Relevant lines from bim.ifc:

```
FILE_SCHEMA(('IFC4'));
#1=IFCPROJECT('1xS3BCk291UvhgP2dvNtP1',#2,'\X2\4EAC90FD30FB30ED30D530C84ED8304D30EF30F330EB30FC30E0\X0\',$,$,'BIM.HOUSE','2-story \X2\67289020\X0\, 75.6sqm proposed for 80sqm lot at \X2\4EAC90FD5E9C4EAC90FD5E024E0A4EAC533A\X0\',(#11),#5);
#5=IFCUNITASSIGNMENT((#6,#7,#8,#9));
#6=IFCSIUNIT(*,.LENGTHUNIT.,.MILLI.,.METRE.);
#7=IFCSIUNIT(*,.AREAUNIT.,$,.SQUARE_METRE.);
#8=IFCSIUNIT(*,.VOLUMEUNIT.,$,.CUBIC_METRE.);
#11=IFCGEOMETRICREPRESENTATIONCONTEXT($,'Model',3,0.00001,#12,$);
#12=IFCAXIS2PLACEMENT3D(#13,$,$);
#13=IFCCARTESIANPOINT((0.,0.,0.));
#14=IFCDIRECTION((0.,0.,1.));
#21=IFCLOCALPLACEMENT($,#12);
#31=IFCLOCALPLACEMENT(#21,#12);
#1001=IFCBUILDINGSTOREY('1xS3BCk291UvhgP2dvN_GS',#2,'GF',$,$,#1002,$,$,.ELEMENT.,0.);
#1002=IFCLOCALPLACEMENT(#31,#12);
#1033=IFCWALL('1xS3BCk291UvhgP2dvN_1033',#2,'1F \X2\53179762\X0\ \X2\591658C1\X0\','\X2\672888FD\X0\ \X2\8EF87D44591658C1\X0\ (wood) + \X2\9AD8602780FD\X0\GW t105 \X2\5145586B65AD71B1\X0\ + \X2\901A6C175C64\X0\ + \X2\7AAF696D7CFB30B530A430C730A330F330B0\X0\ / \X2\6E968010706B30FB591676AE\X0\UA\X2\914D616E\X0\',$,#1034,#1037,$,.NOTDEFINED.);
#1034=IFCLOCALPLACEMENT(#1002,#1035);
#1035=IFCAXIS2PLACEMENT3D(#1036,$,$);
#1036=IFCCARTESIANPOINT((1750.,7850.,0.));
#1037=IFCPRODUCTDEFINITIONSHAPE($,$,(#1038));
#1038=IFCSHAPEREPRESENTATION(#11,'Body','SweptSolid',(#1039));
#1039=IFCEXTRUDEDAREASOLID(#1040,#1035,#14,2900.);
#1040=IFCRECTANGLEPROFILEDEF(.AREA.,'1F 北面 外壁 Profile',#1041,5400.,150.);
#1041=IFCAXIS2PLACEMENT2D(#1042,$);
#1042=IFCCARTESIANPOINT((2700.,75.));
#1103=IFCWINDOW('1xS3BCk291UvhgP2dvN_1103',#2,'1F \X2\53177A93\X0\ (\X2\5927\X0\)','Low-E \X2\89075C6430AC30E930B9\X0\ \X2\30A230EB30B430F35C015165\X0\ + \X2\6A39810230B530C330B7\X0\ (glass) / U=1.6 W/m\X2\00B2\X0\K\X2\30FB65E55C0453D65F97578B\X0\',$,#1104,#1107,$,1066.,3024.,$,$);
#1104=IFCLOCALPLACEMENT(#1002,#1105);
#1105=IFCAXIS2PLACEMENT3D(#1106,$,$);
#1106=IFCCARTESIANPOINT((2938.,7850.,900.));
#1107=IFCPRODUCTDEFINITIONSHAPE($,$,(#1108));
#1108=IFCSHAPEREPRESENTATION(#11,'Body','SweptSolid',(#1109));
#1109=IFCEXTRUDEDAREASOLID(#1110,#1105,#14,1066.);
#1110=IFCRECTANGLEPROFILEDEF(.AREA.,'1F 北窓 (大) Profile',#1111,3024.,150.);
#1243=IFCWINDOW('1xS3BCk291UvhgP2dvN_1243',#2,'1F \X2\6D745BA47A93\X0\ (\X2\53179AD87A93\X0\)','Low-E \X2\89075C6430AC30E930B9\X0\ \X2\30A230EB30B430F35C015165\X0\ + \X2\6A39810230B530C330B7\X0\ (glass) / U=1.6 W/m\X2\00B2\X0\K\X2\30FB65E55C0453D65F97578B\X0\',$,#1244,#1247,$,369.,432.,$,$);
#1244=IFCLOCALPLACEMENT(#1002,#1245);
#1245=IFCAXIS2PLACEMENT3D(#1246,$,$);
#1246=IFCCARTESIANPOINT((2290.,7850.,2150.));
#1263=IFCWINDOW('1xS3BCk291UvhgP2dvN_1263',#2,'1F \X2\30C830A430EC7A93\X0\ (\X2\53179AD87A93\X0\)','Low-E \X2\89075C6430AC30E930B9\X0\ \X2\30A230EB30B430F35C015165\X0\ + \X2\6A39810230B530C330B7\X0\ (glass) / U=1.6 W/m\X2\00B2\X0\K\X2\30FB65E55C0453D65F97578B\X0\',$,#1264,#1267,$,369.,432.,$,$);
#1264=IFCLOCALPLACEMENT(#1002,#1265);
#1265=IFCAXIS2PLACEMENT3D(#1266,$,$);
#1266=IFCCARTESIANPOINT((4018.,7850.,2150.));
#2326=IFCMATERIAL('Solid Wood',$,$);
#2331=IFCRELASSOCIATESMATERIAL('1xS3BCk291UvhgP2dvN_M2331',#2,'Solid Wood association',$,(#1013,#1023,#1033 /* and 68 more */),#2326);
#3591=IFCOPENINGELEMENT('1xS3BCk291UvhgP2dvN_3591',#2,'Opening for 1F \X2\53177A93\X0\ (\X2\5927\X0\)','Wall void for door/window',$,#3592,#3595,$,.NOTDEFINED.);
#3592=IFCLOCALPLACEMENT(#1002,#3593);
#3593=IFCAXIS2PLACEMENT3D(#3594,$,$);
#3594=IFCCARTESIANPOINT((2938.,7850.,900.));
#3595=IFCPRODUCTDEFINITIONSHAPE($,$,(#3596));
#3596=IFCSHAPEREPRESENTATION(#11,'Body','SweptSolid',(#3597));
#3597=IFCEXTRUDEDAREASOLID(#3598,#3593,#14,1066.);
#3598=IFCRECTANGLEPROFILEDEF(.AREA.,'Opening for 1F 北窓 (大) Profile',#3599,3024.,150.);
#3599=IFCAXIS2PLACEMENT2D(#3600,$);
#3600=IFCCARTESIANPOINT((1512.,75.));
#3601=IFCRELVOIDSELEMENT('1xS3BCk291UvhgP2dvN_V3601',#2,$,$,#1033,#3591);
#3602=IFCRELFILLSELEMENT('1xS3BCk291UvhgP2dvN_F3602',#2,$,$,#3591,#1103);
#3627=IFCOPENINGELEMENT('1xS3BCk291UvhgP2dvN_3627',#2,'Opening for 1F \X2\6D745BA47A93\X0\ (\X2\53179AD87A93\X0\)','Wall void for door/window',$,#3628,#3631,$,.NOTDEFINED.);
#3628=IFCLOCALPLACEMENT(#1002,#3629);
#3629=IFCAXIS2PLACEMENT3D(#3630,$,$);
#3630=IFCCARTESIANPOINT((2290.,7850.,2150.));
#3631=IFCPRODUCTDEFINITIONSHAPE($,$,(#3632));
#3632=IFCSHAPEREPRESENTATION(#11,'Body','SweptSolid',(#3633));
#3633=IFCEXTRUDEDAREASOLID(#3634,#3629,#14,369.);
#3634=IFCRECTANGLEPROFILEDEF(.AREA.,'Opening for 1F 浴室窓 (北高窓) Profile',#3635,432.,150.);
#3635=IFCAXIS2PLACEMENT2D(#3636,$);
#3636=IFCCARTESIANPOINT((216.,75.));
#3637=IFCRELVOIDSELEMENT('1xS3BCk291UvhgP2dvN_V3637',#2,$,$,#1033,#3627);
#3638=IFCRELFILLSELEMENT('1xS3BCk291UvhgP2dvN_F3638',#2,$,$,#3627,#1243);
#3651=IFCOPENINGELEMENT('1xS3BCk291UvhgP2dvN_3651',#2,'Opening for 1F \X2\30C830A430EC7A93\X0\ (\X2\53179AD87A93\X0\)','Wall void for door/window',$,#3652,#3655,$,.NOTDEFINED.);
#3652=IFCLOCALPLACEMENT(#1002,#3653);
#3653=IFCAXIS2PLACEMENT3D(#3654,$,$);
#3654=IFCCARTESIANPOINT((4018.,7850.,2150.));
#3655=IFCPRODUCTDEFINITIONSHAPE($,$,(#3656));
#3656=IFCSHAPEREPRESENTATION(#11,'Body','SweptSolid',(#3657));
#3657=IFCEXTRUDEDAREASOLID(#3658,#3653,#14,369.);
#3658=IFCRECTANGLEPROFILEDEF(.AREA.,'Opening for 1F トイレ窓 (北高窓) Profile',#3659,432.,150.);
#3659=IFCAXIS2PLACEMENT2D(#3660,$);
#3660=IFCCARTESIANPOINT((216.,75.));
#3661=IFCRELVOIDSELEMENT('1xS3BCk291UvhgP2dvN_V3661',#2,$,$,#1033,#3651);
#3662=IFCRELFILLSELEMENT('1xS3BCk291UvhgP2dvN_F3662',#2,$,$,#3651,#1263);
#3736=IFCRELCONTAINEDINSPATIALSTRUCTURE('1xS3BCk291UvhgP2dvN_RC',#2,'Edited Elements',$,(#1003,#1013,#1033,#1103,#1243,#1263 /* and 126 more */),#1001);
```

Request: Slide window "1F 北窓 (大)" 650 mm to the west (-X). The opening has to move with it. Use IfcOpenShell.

```python
import ifcopenshell
import ifcopenshell.api.geometry
import ifcopenshell.util.placement
import ifcopenshell.util.unit

model = ifcopenshell.open("bim.ifc")
unit_scale = ifcopenshell.util.unit.calculate_unit_scale(model)

window = model.by_guid("1xS3BCk291UvhgP2dvN_1103")
opening = window.FillsVoids[0].RelatingOpeningElement
wall = opening.VoidsElements[0].RelatingBuildingElement

wall_matrix = ifcopenshell.util.placement.get_local_placement(wall.ObjectPlacement)
shift = wall_matrix[:3, 0] * -0.65 / unit_scale
before = ifcopenshell.util.placement.get_local_placement(window.ObjectPlacement)[:3, 3].copy()

# The window is not placed relative to its opening, so move both.
for product in (opening, window):
    matrix = ifcopenshell.util.placement.get_local_placement(product.ObjectPlacement)
    matrix[:3, 3] += shift
    ifcopenshell.api.geometry.edit_object_placement(model, product=product, matrix=matrix, is_si=False)

after = ifcopenshell.util.placement.get_local_placement(window.ObjectPlacement)[:3, 3]
print("window moved by", (after - before).round(3) + 0.0)

model.write("bim_v2.ifc")
```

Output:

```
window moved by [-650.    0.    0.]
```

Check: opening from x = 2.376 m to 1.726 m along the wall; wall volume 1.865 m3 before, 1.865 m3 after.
